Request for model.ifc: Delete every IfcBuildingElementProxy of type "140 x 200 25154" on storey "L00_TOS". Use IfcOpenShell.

First a look at what the model holds.

```python
import ifcopenshell
import ifcopenshell.util.element

model = ifcopenshell.open("model.ifc")
print(model.schema)
storey = next(s for s in model.by_type("IfcBuildingStorey") if s.Name == "L00_TOS")
proxies = [e for e in ifcopenshell.util.element.get_decomposition(storey) if e.is_a("IfcBuildingElementProxy")]
seen = {}
for e in proxies:
    element_type = ifcopenshell.util.element.get_type(e)
    name = element_type.Name if element_type not in (None, e) else None
    seen[name] = seen.get(name, 0) + 1
for name, count in sorted(seen.items(), key=str):
    print(count, "x", name)
```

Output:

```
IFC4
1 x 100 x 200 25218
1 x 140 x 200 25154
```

```python
import ifcopenshell
import ifcopenshell.api.root
import ifcopenshell.util.element

model = ifcopenshell.open("model.ifc")

storey = next(s for s in model.by_type("IfcBuildingStorey") if s.Name == "L00_TOS")
proxies = [e for e in ifcopenshell.util.element.get_decomposition(storey) if e.is_a("IfcBuildingElementProxy")]
targets = [e for e in proxies if (t := ifcopenshell.util.element.get_type(e)) not in (None, e) and t.Name == "140 x 200 25154"]

for e in targets:
    ifcopenshell.api.root.remove_product(model, product=e)
print(len(targets), "removed")

model.write("model_rev.ifc")
```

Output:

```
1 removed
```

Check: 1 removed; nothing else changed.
